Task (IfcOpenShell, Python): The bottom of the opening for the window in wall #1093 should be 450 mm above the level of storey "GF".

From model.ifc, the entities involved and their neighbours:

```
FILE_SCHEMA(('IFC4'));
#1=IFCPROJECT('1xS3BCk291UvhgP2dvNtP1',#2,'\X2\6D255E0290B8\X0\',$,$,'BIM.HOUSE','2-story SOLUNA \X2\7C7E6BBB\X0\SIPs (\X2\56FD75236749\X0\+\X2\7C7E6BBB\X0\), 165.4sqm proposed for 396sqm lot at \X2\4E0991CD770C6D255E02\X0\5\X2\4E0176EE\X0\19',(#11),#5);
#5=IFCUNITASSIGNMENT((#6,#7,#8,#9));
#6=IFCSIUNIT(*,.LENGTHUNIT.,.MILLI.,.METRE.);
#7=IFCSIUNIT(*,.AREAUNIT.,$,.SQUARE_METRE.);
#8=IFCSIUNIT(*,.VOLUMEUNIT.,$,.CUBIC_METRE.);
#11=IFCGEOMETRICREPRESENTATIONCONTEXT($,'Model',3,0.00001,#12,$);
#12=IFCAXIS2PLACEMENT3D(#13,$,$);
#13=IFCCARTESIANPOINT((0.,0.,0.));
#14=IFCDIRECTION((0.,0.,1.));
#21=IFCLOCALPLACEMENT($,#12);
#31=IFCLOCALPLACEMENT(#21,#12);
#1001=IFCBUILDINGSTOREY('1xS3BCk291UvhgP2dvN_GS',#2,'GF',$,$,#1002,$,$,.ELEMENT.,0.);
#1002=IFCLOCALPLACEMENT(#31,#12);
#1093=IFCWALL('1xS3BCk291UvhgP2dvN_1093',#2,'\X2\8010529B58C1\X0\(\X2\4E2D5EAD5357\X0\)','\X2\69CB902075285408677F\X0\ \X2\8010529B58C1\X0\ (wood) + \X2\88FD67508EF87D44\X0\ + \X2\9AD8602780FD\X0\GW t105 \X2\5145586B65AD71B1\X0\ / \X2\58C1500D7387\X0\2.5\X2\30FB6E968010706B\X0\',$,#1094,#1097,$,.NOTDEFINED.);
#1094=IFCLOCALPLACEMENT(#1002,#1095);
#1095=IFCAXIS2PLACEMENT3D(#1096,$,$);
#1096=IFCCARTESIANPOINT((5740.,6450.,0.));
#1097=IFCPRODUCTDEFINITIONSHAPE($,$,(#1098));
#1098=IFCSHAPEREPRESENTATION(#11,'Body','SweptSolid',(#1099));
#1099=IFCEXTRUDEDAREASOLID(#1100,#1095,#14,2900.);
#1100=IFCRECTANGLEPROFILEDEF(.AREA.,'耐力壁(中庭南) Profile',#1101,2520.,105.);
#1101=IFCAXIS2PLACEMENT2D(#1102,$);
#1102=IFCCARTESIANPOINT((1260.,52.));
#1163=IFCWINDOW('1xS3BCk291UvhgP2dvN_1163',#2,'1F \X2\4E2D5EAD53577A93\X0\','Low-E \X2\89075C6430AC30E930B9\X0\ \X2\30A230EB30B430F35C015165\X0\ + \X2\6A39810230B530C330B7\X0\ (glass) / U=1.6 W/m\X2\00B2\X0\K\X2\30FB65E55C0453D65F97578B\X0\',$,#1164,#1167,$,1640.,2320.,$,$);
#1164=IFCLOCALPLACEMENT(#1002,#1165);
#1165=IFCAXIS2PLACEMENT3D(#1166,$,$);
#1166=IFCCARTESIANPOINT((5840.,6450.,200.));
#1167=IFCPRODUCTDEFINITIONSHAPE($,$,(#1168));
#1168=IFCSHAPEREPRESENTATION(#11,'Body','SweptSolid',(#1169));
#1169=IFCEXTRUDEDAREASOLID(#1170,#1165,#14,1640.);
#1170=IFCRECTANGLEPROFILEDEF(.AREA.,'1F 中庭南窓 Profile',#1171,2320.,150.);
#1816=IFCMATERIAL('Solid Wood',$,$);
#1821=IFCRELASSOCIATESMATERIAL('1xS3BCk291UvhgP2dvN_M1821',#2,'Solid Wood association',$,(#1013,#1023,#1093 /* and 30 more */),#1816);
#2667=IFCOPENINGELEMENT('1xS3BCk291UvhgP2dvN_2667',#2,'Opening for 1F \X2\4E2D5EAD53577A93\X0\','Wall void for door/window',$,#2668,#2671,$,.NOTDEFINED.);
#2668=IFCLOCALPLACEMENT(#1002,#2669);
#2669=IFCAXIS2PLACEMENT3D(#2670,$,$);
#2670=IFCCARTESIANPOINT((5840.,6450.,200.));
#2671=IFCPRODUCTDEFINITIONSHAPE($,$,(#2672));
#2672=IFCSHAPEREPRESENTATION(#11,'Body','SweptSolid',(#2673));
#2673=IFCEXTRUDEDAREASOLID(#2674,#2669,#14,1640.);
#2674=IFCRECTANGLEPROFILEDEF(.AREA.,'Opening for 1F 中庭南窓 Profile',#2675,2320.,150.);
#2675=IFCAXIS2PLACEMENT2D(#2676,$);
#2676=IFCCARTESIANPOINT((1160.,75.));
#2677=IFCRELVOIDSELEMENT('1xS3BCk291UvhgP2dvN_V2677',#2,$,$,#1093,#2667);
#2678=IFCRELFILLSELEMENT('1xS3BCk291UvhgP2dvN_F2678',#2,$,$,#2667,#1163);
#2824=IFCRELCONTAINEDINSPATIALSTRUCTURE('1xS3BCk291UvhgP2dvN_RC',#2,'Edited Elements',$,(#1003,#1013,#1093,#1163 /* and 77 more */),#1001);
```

```python
import numpy as np
import ifcopenshell
import ifcopenshell.api.geometry
import ifcopenshell.geom
import ifcopenshell.util.element
import ifcopenshell.util.placement
import ifcopenshell.util.shape
import ifcopenshell.util.unit

model = ifcopenshell.open("model.ifc")
unit_scale = ifcopenshell.util.unit.calculate_unit_scale(model)

window = model.by_id(1163)
opening = window.FillsVoids[0].RelatingOpeningElement
storey = ifcopenshell.util.element.get_container(window, ifc_class="IfcBuildingStorey")
level = ifcopenshell.util.placement.get_local_placement(storey.ObjectPlacement)[2, 3]

# The opening's origin need not be at the sill, so measure its lowest point.
shape = ifcopenshell.geom.create_shape(ifcopenshell.geom.settings(), opening)
bottom = ifcopenshell.util.shape.get_shape_bottom_elevation(shape, shape.geometry) / unit_scale
dz = level + 450.0 - bottom

shift = np.array([0.0, 0.0, dz])
# The window is not placed relative to its opening, so move both.
for product in (opening, window):
    matrix = ifcopenshell.util.placement.get_local_placement(product.ObjectPlacement)
    matrix[:3, 3] += shift
    ifcopenshell.api.geometry.edit_object_placement(model, product=product, matrix=matrix, is_si=False)

print(f"moved by {dz * unit_scale:+.3f} m")

model.write("model-out.ifc")
```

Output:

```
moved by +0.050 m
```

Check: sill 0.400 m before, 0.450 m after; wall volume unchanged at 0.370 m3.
